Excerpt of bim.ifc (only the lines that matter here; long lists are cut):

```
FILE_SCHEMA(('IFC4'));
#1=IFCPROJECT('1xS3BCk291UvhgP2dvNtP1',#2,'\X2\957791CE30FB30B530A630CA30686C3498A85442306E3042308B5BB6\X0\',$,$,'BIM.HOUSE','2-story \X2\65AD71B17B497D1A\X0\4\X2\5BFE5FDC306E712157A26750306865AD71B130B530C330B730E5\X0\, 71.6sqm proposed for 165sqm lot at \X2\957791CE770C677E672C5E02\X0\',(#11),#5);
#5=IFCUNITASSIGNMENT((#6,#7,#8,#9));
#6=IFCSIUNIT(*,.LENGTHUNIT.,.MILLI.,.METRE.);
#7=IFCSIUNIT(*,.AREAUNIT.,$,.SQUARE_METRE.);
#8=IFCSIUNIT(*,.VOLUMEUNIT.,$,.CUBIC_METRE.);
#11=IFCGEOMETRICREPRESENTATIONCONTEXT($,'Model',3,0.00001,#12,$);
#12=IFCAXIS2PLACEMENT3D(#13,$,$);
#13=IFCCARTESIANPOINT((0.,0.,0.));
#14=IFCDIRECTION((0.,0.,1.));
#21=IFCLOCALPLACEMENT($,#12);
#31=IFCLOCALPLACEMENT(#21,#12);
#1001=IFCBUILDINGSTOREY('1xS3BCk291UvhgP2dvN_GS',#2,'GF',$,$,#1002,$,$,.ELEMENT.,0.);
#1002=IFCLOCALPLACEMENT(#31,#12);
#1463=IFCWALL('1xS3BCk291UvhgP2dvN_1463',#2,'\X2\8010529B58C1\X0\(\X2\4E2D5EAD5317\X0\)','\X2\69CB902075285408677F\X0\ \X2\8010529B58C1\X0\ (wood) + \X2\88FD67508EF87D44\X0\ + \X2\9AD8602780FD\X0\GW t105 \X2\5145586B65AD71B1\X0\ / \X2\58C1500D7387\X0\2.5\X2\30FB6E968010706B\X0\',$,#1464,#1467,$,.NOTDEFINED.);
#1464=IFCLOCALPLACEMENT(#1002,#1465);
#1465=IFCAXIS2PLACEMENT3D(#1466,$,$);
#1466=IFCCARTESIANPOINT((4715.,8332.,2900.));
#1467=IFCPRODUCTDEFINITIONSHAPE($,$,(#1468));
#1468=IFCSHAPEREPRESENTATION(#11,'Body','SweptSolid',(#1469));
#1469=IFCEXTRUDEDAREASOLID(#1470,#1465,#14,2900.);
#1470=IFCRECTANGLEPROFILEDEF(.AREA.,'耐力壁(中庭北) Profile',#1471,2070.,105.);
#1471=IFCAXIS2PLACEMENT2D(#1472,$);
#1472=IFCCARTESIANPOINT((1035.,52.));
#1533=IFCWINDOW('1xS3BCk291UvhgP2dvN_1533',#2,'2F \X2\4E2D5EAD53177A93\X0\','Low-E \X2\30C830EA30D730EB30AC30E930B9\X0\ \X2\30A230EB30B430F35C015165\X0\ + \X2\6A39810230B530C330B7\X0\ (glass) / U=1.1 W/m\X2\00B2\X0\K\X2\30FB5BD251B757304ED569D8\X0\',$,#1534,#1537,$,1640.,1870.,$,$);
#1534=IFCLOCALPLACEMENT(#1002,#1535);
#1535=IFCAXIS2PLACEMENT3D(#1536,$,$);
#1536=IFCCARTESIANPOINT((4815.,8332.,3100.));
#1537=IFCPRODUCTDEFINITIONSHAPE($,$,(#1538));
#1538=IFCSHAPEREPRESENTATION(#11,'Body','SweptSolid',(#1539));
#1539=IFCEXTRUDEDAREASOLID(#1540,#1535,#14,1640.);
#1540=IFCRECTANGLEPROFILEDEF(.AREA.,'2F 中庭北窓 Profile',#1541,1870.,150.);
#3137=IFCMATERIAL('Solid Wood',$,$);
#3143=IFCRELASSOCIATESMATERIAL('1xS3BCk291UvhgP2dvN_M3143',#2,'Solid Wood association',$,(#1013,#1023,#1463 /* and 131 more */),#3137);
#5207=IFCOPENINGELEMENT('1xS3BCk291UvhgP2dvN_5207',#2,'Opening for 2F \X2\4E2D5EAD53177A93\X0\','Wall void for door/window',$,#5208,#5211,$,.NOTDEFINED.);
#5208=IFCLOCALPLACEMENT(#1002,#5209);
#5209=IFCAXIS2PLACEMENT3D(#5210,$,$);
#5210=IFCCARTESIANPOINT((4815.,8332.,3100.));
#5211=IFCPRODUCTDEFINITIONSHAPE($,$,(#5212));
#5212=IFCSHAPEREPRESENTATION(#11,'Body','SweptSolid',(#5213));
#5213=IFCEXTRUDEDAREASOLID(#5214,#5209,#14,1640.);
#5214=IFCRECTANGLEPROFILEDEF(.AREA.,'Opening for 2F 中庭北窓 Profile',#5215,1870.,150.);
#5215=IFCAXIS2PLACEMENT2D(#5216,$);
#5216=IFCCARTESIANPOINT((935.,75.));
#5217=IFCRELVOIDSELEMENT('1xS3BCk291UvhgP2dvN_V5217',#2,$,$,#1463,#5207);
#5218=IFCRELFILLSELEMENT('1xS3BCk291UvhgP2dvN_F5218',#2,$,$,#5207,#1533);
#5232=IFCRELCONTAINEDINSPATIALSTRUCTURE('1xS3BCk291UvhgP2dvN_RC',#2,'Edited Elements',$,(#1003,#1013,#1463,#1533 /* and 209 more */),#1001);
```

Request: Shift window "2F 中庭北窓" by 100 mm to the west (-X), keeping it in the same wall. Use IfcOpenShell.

```python
import ifcopenshell
import ifcopenshell.api.geometry
import ifcopenshell.util.placement

model = ifcopenshell.open("bim.ifc")

window = model.by_guid("1xS3BCk291UvhgP2dvN_1533")
opening = window.FillsVoids[0].RelatingOpeningElement
wall = opening.VoidsElements[0].RelatingBuildingElement

wall_matrix = ifcopenshell.util.placement.get_local_placement(wall.ObjectPlacement)
shift = wall_matrix[:3, 0] * -100.0
before = ifcopenshell.util.placement.get_local_placement(window.ObjectPlacement)[:3, 3].copy()

# The window is not placed relative to its opening, so move both.
for product in (opening, window):
    matrix = ifcopenshell.util.placement.get_local_placement(product.ObjectPlacement)
    matrix[:3, 3] += shift
    ifcopenshell.api.geometry.edit_object_placement(model, product=product, matrix=matrix, is_si=False)

after = ifcopenshell.util.placement.get_local_placement(window.ObjectPlacement)[:3, 3]
print("window moved by", (after - before).round(3) + 0.0)

model.write("bim-out.ifc")
```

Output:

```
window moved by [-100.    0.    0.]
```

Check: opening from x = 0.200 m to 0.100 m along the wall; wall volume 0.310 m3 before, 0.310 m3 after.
